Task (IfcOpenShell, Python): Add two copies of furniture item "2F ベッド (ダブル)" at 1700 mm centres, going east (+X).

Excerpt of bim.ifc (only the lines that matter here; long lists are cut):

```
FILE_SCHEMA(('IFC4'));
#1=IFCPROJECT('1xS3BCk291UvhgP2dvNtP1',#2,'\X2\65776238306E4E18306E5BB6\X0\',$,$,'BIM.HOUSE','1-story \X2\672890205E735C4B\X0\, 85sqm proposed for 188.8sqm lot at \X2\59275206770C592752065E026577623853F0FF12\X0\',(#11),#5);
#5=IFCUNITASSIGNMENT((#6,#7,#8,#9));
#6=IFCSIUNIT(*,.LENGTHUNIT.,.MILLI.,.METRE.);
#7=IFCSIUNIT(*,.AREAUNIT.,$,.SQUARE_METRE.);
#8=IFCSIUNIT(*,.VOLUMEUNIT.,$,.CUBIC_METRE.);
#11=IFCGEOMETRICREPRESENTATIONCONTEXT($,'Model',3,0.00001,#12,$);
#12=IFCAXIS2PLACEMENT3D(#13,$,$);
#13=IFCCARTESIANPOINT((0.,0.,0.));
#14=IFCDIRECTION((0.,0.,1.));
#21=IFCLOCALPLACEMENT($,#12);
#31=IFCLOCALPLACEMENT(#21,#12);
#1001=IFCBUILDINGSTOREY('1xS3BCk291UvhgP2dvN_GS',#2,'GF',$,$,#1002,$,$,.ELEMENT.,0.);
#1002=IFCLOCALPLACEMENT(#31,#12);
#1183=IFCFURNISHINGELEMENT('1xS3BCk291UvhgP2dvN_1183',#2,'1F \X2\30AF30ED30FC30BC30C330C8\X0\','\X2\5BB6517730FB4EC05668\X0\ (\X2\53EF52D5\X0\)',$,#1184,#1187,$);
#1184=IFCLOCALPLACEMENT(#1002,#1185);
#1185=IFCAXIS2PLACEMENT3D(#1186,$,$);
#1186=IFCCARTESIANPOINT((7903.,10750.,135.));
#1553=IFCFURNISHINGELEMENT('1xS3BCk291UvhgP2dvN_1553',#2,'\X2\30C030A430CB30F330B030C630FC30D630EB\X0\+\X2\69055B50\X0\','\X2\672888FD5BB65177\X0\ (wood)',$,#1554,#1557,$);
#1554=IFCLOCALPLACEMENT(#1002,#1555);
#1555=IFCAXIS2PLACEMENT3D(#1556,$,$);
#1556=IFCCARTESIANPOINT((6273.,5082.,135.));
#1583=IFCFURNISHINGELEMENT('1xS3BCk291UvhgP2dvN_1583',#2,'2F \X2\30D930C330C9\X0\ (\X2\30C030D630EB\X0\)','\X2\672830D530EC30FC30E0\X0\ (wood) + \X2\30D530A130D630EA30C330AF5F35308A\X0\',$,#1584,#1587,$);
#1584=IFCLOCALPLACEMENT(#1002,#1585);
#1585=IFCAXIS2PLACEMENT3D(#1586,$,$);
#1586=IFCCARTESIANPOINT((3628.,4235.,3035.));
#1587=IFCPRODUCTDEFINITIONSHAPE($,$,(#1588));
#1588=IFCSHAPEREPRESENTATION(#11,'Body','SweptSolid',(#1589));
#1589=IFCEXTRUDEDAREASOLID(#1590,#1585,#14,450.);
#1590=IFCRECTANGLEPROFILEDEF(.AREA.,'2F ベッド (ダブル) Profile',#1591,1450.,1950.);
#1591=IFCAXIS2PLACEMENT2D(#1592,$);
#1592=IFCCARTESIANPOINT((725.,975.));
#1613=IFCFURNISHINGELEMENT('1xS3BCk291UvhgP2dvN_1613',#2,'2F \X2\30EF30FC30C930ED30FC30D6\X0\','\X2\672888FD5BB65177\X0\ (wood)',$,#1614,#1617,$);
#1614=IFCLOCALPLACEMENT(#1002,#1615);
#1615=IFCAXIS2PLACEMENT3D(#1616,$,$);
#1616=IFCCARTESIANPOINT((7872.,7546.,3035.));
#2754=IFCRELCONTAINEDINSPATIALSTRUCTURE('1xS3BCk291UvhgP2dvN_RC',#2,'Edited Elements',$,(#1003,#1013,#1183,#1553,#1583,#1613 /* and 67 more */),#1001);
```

```python
import numpy as np
import ifcopenshell
import ifcopenshell.api.geometry
import ifcopenshell.api.root
import ifcopenshell.util.element
import ifcopenshell.util.placement
import ifcopenshell.util.unit

model = ifcopenshell.open("bim.ifc")
unit_scale = ifcopenshell.util.unit.calculate_unit_scale(model)


def reuse_history(source, copy):
    """copy_class also copies each property set's owner history, people and application; keep the originals."""
    for rel in copy.IsDefinedBy:
        if rel.is_a("IfcRelDefinesByProperties") and (history := rel.RelatingPropertyDefinition.OwnerHistory):
            rel.RelatingPropertyDefinition.OwnerHistory = source.OwnerHistory
            ifcopenshell.util.element.remove_deep2(model, history)


source = model.by_guid("1xS3BCk291UvhgP2dvN_1583")
base = ifcopenshell.util.placement.get_local_placement(source.ObjectPlacement)
step = np.array([1.0, 0.0, 0.0]) * 1.7 / unit_scale

for i in range(1, 3):
    copy = ifcopenshell.api.root.copy_class(model, product=source)
    copy.Representation = ifcopenshell.util.element.copy_deep(
        model, source.Representation, exclude=["IfcGeometricRepresentationContext", "IfcRepresentationMap"]
    )
    reuse_history(source, copy)
    matrix = base.copy()
    matrix[:3, 3] += i * step
    print("added at", matrix[:3, 3].round(3) + 0.0)
    ifcopenshell.api.geometry.edit_object_placement(model, product=copy, matrix=matrix, is_si=False)

model.write("bim_edited.ifc")
```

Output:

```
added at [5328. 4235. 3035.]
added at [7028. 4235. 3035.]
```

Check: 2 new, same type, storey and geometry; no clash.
